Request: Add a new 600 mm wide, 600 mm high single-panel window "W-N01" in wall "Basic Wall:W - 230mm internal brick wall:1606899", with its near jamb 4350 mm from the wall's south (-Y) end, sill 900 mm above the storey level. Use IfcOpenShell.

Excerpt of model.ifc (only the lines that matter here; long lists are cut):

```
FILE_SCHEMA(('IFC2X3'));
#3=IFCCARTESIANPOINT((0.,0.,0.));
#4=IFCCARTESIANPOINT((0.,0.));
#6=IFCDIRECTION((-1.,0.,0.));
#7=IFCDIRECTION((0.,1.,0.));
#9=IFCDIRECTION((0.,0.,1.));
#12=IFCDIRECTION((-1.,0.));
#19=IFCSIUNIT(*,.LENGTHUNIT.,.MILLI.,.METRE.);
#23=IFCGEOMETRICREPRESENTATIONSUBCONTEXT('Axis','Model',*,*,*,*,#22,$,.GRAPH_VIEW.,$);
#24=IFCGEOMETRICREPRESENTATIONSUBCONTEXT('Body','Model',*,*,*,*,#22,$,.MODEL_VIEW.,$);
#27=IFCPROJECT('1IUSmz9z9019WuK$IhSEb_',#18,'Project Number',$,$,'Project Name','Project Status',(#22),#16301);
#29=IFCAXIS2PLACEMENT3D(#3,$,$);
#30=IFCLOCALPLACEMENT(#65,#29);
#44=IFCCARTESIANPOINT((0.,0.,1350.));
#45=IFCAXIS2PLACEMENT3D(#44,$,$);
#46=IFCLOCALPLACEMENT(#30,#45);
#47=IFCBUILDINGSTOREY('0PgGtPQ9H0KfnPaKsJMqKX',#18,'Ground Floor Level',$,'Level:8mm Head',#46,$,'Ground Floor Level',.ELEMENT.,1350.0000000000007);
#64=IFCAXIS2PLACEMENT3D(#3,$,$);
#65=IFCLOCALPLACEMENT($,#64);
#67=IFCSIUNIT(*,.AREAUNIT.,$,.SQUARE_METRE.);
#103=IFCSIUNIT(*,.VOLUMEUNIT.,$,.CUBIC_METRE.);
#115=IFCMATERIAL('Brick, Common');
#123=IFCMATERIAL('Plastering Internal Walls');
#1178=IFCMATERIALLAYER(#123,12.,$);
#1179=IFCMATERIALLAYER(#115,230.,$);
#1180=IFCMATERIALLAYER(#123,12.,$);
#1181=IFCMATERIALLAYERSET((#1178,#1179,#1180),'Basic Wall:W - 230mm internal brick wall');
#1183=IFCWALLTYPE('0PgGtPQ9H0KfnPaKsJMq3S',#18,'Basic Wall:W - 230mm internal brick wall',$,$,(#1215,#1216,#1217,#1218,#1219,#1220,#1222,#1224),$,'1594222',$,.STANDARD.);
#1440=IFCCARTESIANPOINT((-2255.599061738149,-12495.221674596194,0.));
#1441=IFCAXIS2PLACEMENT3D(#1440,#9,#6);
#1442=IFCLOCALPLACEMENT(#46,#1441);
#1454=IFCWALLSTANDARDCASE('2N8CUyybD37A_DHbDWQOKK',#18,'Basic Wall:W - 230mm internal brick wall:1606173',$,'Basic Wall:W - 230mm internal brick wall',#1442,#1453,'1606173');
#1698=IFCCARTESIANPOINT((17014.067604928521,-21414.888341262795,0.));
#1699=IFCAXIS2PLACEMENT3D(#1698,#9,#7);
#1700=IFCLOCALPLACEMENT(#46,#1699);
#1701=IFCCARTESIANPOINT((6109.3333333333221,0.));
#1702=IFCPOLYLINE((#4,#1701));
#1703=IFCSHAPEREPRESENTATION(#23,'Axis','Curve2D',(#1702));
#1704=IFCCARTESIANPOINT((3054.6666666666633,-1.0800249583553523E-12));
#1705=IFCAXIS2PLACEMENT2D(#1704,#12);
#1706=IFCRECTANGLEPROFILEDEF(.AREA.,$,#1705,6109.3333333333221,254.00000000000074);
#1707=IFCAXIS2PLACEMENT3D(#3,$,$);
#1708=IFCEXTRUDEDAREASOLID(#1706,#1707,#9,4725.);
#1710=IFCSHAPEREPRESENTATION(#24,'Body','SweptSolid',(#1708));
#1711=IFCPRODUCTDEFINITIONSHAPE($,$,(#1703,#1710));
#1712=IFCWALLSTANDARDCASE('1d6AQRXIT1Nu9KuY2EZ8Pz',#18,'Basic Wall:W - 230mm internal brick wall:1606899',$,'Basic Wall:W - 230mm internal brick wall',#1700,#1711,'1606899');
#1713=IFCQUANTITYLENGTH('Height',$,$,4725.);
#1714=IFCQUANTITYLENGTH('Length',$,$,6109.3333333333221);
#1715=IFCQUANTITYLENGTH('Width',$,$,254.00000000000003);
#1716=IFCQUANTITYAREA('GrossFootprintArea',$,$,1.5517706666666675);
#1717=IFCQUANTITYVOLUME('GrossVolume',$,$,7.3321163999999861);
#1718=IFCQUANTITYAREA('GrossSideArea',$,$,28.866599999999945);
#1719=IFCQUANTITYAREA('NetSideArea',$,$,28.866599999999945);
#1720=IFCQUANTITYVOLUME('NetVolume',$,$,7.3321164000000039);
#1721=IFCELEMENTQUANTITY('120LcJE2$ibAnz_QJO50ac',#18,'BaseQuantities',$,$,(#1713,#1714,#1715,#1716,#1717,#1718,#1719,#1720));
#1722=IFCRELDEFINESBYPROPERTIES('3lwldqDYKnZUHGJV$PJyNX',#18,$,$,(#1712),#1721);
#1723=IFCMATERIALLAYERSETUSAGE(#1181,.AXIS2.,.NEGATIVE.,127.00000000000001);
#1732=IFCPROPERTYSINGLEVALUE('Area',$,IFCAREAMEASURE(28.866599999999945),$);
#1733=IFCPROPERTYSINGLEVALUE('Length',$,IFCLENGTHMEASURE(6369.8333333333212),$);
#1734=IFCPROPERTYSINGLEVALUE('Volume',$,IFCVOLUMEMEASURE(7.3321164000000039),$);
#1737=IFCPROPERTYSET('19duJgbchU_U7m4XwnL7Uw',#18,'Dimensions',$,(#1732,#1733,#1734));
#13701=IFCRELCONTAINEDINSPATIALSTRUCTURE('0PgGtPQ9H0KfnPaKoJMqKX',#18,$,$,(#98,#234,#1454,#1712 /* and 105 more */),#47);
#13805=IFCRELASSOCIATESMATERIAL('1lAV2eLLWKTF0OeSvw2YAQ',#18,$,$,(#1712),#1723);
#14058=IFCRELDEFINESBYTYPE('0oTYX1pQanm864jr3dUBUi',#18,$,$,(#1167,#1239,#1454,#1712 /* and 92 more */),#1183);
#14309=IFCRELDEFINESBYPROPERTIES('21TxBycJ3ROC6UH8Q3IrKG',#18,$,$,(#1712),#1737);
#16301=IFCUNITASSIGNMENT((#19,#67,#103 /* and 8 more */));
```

```python
import numpy as np
import ifcopenshell
import ifcopenshell.api.feature
import ifcopenshell.api.geometry
import ifcopenshell.api.pset
import ifcopenshell.api.root
import ifcopenshell.api.spatial
import ifcopenshell.api.type
import ifcopenshell.geom
import ifcopenshell.util.element
import ifcopenshell.util.placement
import ifcopenshell.util.representation
import ifcopenshell.util.shape
import ifcopenshell.util.unit

model = ifcopenshell.open("model.ifc")
unit_scale = ifcopenshell.util.unit.calculate_unit_scale(model)
area_scale = ifcopenshell.util.unit.calculate_unit_scale(model, "AREAUNIT")
volume_scale = ifcopenshell.util.unit.calculate_unit_scale(model, "VOLUMEUNIT")
settings = ifcopenshell.geom.settings()


def volume(element):
    """Net volume in cubic metres, openings subtracted."""
    shape = ifcopenshell.geom.create_shape(settings, element)
    return ifcopenshell.util.shape.get_volume(shape.geometry)


wall = model.by_guid("1d6AQRXIT1Nu9KuY2EZ8Pz")
storey = ifcopenshell.util.element.get_container(wall, ifc_class="IfcBuildingStorey")
context = ifcopenshell.util.representation.get_context(model, "Model", "Body", "MODEL_VIEW")
before = volume(wall)

width, height, from_end, sill = 0.6, 0.6, 4.35, 0.9  # metres

# The wall runs along its own X axis, and the end named is its -X end.
wall_shape = ifcopenshell.geom.create_shape(settings, wall)
x, y, z = ifcopenshell.util.shape.get_vertices(wall_shape.geometry).T
start = x.min() + from_end
face, thickness = float(y.min()), float(y.max() - y.min())
wall_matrix = ifcopenshell.util.placement.get_local_placement(wall.ObjectPlacement)
level = ifcopenshell.util.placement.get_local_placement(storey.ObjectPlacement)[2, 3]


def in_wall(x, y):
    """Placement at x, y metres in the wall's axes, at sill height."""
    matrix = wall_matrix.copy()
    matrix[:, 3] = wall_matrix @ np.array([x / unit_scale, y / unit_scale, 0.0, 1.0])
    matrix[2, 3] = level + sill / unit_scale
    return matrix


# Opening: a box that overshoots both wall faces by 50 mm.
opening = ifcopenshell.api.root.create_entity(model, ifc_class="IfcOpeningElement")
box = ifcopenshell.api.geometry.add_wall_representation(
    model, context=context, length=width, height=height, thickness=thickness + 0.1
)
ifcopenshell.api.geometry.assign_representation(model, product=opening, representation=box)
ifcopenshell.api.geometry.edit_object_placement(model, product=opening, matrix=in_wall(start, face - 0.05), is_si=False)
ifcopenshell.api.feature.add_feature(model, feature=opening, element=wall)

window = ifcopenshell.api.root.create_entity(model, ifc_class="IfcWindow", name="W-N01")
window.OverallWidth, window.OverallHeight = width / unit_scale, height / unit_scale
body = ifcopenshell.api.geometry.add_window_representation(
    model,
    context=context,
    overall_width=window.OverallWidth,
    overall_height=window.OverallHeight,
    partition_type="SINGLE_PANEL",
)
ifcopenshell.api.geometry.assign_representation(model, product=window, representation=body)
ifcopenshell.api.spatial.assign_container(model, products=[window], relating_structure=storey)
fills = ifcopenshell.api.feature.add_filling(model, opening=opening, element=window)
fills.OwnerHistory = window.OwnerHistory  # required in IFC2X3

# IFC2X3 keeps the operation on the window style.
style = ifcopenshell.api.root.create_entity(model, ifc_class="IfcWindowStyle", name="W-N01")
style.OperationType, style.ConstructionType = "SINGLE_PANEL", "NOTDEFINED"
style.ParameterTakesPrecedence = style.Sizeable = False
ifcopenshell.api.type.assign_type(model, related_objects=[window], relating_type=style)

# Centre the window in the wall's thickness.
ifcopenshell.api.geometry.edit_object_placement(model, product=window, matrix=in_wall(start, face), is_si=False)
window_shape = ifcopenshell.geom.create_shape(settings, window)
depth = ifcopenshell.util.shape.get_vertices(window_shape.geometry)[:, 1]
offset = face + thickness / 2 - (depth.min() + depth.max()) / 2
ifcopenshell.api.geometry.edit_object_placement(model, product=window, matrix=in_wall(start, offset), is_si=False)

after = volume(wall)

# Update the wall's stored quantities.
qto = model.by_id(ifcopenshell.util.element.get_pset(wall, "BaseQuantities", should_inherit=False)["id"])
ifcopenshell.api.pset.edit_qto(model, qto=qto, properties={
    "NetSideArea": after / thickness / area_scale,
    "NetVolume": after / volume_scale,
})
pset = model.by_id(ifcopenshell.util.element.get_pset(wall, "Dimensions", should_inherit=False)["id"])
ifcopenshell.api.pset.edit_pset(model, pset=pset, properties={
    "Area": model.create_entity("IfcAreaMeasure", after / thickness / area_scale),
    "Volume": model.create_entity("IfcVolumeMeasure", after / volume_scale),
})

print(f"wall volume {before:.3f} -> {after:.3f} m3")

model.write("model_v2.ifc")
```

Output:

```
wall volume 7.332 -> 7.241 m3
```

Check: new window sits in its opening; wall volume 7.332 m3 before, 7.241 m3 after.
